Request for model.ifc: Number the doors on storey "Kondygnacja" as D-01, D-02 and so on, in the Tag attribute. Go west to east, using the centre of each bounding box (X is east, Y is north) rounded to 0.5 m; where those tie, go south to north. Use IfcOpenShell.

First a look at what the model holds.

```python
import ifcopenshell
import ifcopenshell.util.element
import ifcopenshell.util.placement

model = ifcopenshell.open("model.ifc")
print(model.schema)
storey = next(s for s in model.by_type("IfcBuildingStorey") if s.Name == "Kondygnacja")
doors = [e for e in ifcopenshell.util.element.get_decomposition(storey) if e.is_a("IfcDoor")]
for e in sorted(doors, key=lambda e: e.id()):
    origin = ifcopenshell.util.placement.get_local_placement(e.ObjectPlacement)[:3, 3]
    print(e.id(), e.Tag, e.Name, origin.round(2) + 0.0, sep=" | ")
```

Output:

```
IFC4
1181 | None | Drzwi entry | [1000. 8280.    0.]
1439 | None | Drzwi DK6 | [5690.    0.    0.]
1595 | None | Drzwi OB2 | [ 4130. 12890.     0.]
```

```python
import ifcopenshell
import ifcopenshell.geom
import ifcopenshell.util.element
import ifcopenshell.util.shape

model = ifcopenshell.open("model.ifc")
settings = ifcopenshell.geom.settings()
settings.set("use-world-coords", True)


def centre(element):
    shape = ifcopenshell.geom.create_shape(settings, element)
    return ifcopenshell.util.shape.get_bbox_centroid(shape.geometry)


storey = next(s for s in model.by_type("IfcBuildingStorey") if s.Name == "Kondygnacja")
doors = [e for e in ifcopenshell.util.element.get_decomposition(storey) if e.is_a("IfcDoor")]

# Insertion points can sit at a corner or the storey origin, so sort by the geometry (in metres).
centres = {e: centre(e) for e in doors}
doors.sort(key=lambda e: (round(centres[e][0] / 0.5), centres[e][1]))

for i, e in enumerate(doors, start=1):
    number = f"D-{i:02d}"
    e.Tag = number
    print(e.id(), number)

model.write("model_edited.ifc")
```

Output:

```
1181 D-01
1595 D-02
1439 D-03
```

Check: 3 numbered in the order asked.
